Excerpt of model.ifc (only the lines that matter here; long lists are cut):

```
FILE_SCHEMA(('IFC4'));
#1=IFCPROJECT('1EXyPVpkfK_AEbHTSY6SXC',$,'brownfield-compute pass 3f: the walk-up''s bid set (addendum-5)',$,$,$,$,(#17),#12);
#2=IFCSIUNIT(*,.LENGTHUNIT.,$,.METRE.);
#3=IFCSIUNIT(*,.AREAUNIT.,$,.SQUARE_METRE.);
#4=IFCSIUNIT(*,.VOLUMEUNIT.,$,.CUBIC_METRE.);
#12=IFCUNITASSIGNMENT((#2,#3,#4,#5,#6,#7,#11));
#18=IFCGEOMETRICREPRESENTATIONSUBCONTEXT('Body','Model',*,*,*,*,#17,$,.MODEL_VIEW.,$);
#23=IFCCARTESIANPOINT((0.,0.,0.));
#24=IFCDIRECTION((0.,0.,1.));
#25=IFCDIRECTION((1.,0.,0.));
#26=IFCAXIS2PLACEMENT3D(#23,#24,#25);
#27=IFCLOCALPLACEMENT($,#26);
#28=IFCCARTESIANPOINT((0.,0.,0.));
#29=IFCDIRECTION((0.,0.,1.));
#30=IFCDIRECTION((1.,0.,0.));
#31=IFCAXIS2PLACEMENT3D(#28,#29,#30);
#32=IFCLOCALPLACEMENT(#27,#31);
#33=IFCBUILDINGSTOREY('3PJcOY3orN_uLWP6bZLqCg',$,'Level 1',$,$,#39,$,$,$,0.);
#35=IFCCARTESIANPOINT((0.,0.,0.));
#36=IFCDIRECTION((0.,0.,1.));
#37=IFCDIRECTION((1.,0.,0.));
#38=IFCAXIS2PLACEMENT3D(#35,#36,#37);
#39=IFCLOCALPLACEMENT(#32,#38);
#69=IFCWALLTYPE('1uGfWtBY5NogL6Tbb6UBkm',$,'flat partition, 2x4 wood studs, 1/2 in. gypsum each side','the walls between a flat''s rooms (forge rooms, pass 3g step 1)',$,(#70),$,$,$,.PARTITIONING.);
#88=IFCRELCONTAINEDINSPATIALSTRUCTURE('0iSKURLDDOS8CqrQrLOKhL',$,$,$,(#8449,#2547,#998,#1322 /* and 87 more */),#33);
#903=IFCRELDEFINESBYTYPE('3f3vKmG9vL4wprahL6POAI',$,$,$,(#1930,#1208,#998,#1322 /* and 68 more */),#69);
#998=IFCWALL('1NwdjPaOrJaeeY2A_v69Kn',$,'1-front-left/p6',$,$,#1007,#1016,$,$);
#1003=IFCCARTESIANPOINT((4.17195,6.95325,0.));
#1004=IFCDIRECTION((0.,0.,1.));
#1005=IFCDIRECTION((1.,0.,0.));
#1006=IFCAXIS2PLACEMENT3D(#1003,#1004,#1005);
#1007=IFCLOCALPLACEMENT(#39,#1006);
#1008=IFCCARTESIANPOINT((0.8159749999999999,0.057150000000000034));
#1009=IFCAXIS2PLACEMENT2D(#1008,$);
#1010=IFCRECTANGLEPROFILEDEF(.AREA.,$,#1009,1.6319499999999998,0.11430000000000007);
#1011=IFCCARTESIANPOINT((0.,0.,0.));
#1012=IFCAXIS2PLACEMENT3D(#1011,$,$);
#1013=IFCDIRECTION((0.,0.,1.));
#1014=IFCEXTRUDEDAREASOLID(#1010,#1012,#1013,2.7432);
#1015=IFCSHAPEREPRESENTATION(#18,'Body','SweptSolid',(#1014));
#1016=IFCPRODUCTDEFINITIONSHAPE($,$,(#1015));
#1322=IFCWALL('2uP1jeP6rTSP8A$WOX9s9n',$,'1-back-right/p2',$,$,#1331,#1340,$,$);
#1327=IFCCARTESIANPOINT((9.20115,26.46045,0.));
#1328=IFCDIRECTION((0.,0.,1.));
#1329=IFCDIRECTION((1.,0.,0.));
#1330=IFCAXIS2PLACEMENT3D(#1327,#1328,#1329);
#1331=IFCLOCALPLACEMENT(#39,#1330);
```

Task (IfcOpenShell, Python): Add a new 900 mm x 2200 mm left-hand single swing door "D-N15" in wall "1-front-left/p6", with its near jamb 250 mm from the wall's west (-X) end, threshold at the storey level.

```python
import numpy as np
import ifcopenshell
import ifcopenshell.api.feature
import ifcopenshell.api.geometry
import ifcopenshell.api.root
import ifcopenshell.api.spatial
import ifcopenshell.geom
import ifcopenshell.util.element
import ifcopenshell.util.placement
import ifcopenshell.util.representation
import ifcopenshell.util.shape
import ifcopenshell.util.unit

model = ifcopenshell.open("model.ifc")
unit_scale = ifcopenshell.util.unit.calculate_unit_scale(model)
settings = ifcopenshell.geom.settings()


def volume(element):
    """Net volume in cubic metres, openings subtracted."""
    shape = ifcopenshell.geom.create_shape(settings, element)
    return ifcopenshell.util.shape.get_volume(shape.geometry)


wall = model.by_guid("1NwdjPaOrJaeeY2A_v69Kn")
storey = ifcopenshell.util.element.get_container(wall, ifc_class="IfcBuildingStorey")
context = ifcopenshell.util.representation.get_context(model, "Model", "Body", "MODEL_VIEW")
before = volume(wall)

width, height, from_end, sill = 0.9, 2.2, 0.25, 0.0  # metres

# The wall runs along its own X axis, and the end named is its -X end.
wall_shape = ifcopenshell.geom.create_shape(settings, wall)
x, y, z = ifcopenshell.util.shape.get_vertices(wall_shape.geometry).T
start = x.min() + from_end
face, thickness = float(y.min()), float(y.max() - y.min())
wall_matrix = ifcopenshell.util.placement.get_local_placement(wall.ObjectPlacement)
level = ifcopenshell.util.placement.get_local_placement(storey.ObjectPlacement)[2, 3]


def in_wall(x, y):
    """Placement at x, y metres in the wall's axes, at sill height."""
    matrix = wall_matrix.copy()
    matrix[:, 3] = wall_matrix @ np.array([x / unit_scale, y / unit_scale, 0.0, 1.0])
    matrix[2, 3] = level + sill / unit_scale
    return matrix


# Opening: a box that overshoots both wall faces by 50 mm.
opening = ifcopenshell.api.root.create_entity(model, ifc_class="IfcOpeningElement", predefined_type="OPENING")
box = ifcopenshell.api.geometry.add_wall_representation(
    model, context=context, length=width, height=height, thickness=thickness + 0.1
)
ifcopenshell.api.geometry.assign_representation(model, product=opening, representation=box)
ifcopenshell.api.geometry.edit_object_placement(model, product=opening, matrix=in_wall(start, face - 0.05), is_si=False)
ifcopenshell.api.feature.add_feature(model, feature=opening, element=wall)

door = ifcopenshell.api.root.create_entity(model, ifc_class="IfcDoor", name="D-N15", predefined_type="DOOR")
door.OverallWidth, door.OverallHeight = width / unit_scale, height / unit_scale
door.OperationType = "SINGLE_SWING_LEFT"
body = ifcopenshell.api.geometry.add_door_representation(
    model,
    context=context,
    overall_width=door.OverallWidth,
    overall_height=door.OverallHeight,
    operation_type="SINGLE_SWING_LEFT",
    lining_properties={"LiningDepth": thickness / unit_scale, "ThresholdDepth": thickness / unit_scale},
)
ifcopenshell.api.geometry.assign_representation(model, product=door, representation=body)
ifcopenshell.api.spatial.assign_container(model, products=[door], relating_structure=storey)
ifcopenshell.api.feature.add_filling(model, opening=opening, element=door)

# The lining spans the wall, so the door starts at the wall face.
ifcopenshell.api.geometry.edit_object_placement(model, product=door, matrix=in_wall(start, face), is_si=False)

after = volume(wall)

print(f"wall volume {before:.3f} -> {after:.3f} m3")

model.write("model_updated.ifc")
```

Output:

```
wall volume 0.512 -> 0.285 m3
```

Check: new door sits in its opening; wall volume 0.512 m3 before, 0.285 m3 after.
